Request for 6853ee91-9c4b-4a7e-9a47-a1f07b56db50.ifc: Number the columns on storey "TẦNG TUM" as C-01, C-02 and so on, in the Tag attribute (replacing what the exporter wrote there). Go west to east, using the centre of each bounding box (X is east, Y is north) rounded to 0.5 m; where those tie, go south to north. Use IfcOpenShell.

First a look at what the model holds.

```python
import ifcopenshell
import ifcopenshell.util.element
import ifcopenshell.util.placement

model = ifcopenshell.open("6853ee91-9c4b-4a7e-9a47-a1f07b56db50.ifc")
print(model.schema)
storey = next(s for s in model.by_type("IfcBuildingStorey") if s.Name == "TẦNG TUM")
columns = [e for e in ifcopenshell.util.element.get_decomposition(storey) if e.is_a("IfcColumn")]
for e in sorted(columns, key=lambda e: e.id()):
    origin = ifcopenshell.util.placement.get_local_placement(e.ObjectPlacement)[:3, 3]
    print(e.id(), e.Tag, e.Name, origin.round(2) + 0.0, sep=" | ")
```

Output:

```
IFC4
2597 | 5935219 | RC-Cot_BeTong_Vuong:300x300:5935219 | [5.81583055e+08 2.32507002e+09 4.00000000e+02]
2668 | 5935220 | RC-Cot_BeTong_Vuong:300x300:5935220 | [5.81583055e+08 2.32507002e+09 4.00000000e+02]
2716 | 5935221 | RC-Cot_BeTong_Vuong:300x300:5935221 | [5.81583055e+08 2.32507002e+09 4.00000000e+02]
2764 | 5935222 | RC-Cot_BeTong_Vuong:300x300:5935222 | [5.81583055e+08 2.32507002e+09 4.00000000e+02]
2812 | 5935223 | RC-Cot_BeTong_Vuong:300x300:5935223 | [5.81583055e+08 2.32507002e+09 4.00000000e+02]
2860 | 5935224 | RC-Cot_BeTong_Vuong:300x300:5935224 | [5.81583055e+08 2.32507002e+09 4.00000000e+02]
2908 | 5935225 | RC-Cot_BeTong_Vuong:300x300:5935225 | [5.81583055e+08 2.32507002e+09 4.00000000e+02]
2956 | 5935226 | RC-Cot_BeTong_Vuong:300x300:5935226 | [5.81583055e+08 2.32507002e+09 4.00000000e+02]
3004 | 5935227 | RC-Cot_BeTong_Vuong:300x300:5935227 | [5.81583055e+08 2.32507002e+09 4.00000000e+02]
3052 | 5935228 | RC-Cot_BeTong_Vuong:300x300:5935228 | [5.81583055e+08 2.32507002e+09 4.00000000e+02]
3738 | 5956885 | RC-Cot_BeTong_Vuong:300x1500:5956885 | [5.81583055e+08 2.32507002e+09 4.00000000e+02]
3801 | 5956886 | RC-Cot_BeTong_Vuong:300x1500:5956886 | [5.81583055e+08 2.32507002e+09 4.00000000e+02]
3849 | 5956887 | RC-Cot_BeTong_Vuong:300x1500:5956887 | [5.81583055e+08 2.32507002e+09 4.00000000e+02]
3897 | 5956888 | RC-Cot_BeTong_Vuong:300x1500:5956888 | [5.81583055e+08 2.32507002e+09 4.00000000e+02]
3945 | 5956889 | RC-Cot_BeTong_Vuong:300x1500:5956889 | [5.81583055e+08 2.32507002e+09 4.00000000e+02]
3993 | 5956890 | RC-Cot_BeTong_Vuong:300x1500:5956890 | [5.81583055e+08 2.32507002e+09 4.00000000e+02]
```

```python
import ifcopenshell
import ifcopenshell.geom
import ifcopenshell.util.element
import ifcopenshell.util.shape

model = ifcopenshell.open("6853ee91-9c4b-4a7e-9a47-a1f07b56db50.ifc")
settings = ifcopenshell.geom.settings()
settings.set("use-world-coords", True)


def centre(element):
    shape = ifcopenshell.geom.create_shape(settings, element)
    return ifcopenshell.util.shape.get_bbox_centroid(shape.geometry)


storey = next(s for s in model.by_type("IfcBuildingStorey") if s.Name == "TẦNG TUM")
columns = [e for e in ifcopenshell.util.element.get_decomposition(storey) if e.is_a("IfcColumn")]

# Insertion points can sit at a corner or the storey origin, so sort by the geometry (in metres).
centres = {e: centre(e) for e in columns}
columns.sort(key=lambda e: (round(centres[e][0] / 0.5), centres[e][1]))

for i, e in enumerate(columns, start=1):
    number = f"C-{i:02d}"
    e.Tag = number
    print(e.id(), number)

model.write("6853ee91-9c4b-4a7e-9a47-a1f07b56db50-out.ifc")
```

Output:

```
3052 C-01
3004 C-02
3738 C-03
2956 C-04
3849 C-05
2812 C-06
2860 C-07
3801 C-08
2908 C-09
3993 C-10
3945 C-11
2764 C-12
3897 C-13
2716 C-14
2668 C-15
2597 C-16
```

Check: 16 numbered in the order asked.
